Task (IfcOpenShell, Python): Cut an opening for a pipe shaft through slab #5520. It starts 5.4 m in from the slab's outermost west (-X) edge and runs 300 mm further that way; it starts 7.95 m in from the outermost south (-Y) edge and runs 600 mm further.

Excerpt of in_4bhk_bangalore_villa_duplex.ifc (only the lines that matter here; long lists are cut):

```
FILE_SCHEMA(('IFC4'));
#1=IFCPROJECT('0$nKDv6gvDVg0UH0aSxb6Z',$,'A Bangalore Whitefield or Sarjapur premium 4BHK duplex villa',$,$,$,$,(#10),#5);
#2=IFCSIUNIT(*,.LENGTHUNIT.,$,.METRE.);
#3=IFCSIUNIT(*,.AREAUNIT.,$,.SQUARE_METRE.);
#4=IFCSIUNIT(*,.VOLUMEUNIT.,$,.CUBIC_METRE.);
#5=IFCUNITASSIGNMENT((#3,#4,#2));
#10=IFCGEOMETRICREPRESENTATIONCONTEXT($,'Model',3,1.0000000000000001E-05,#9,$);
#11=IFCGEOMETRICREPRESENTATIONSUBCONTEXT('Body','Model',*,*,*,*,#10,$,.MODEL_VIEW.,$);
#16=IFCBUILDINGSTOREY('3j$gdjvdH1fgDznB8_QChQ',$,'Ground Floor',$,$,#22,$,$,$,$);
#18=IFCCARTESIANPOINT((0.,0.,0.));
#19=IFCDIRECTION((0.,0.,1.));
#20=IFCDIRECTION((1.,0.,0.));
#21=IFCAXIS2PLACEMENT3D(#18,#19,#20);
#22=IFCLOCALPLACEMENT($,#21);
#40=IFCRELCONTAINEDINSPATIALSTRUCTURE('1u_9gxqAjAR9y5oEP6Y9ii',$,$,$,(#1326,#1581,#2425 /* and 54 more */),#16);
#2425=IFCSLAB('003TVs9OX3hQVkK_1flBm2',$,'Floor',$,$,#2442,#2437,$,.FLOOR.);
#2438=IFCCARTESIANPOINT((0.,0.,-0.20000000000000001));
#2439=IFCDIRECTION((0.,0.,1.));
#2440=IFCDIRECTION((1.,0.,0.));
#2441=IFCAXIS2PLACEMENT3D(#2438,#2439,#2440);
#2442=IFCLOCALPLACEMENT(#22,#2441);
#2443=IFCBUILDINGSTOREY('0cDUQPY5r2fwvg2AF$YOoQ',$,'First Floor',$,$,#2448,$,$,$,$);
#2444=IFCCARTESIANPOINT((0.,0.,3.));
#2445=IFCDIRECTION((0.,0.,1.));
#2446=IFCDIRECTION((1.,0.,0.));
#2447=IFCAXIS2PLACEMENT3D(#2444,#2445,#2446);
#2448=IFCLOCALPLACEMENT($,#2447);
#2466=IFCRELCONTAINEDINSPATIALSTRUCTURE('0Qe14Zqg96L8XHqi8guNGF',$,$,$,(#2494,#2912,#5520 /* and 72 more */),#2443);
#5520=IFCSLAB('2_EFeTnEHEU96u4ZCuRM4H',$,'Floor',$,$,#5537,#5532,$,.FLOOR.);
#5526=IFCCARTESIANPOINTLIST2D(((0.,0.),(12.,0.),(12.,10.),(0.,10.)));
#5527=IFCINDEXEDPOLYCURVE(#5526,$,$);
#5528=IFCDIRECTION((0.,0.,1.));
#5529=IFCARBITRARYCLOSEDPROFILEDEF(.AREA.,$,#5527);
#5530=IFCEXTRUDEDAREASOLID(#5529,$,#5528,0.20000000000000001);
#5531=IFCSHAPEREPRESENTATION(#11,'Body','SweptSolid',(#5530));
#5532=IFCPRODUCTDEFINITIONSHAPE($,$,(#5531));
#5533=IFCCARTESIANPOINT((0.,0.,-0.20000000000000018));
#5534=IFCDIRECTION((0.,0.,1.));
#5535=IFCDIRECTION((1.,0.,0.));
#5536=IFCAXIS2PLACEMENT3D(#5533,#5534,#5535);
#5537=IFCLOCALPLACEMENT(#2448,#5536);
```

```python
import numpy as np
import ifcopenshell
import ifcopenshell.api.feature
import ifcopenshell.api.geometry
import ifcopenshell.api.root
import ifcopenshell.geom
import ifcopenshell.util.placement
import ifcopenshell.util.representation
import ifcopenshell.util.shape
import ifcopenshell.util.unit

model = ifcopenshell.open("in_4bhk_bangalore_villa_duplex.ifc")
unit_scale = ifcopenshell.util.unit.calculate_unit_scale(model)
settings = ifcopenshell.geom.settings()


def volume(element):
    """Net volume in cubic metres, openings subtracted."""
    shape = ifcopenshell.geom.create_shape(settings, element)
    return ifcopenshell.util.shape.get_volume(shape.geometry)


slab = model.by_guid("2_EFeTnEHEU96u4ZCuRM4H")
before = volume(slab)

# Extent in the slab's own axes, in metres. The edges named are its -X and -Y sides.
slab_shape = ifcopenshell.geom.create_shape(settings, slab)
vertices = ifcopenshell.util.shape.get_vertices(slab_shape.geometry)
x_min, y_min, bottom = vertices.min(axis=0)
top = vertices[:, 2].max()

opening = ifcopenshell.api.root.create_entity(model, ifc_class="IfcOpeningElement", name="Pipe shaft opening", predefined_type="OPENING")
context = ifcopenshell.util.representation.get_context(model, "Model", "Body", "MODEL_VIEW")
width, depth = 0.3, 0.6
outline = [(0.0, 0.0), (width, 0.0), (width, depth), (0.0, depth), (0.0, 0.0)]
# Overshoot both faces by 50 mm so the cut is clean.
shape = ifcopenshell.api.geometry.add_slab_representation(
    model, context=context, depth=top - bottom + 0.1, polyline=outline
)
ifcopenshell.api.geometry.assign_representation(model, product=opening, representation=shape)

matrix = ifcopenshell.util.placement.get_local_placement(slab.ObjectPlacement)
matrix[:, 3] = matrix @ np.append(np.array([x_min + 5.4, y_min + 7.95, bottom - 0.05]) / unit_scale, 1.0)
ifcopenshell.api.geometry.edit_object_placement(model, product=opening, matrix=matrix, is_si=False)
ifcopenshell.api.feature.add_feature(model, feature=opening, element=slab)

after = volume(slab)

print(f"slab volume {before:.3f} -> {after:.3f} m3")

model.write("in_4bhk_bangalore_villa_duplex-out.ifc")
```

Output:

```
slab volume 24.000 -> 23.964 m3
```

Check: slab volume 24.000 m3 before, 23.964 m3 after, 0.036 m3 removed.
